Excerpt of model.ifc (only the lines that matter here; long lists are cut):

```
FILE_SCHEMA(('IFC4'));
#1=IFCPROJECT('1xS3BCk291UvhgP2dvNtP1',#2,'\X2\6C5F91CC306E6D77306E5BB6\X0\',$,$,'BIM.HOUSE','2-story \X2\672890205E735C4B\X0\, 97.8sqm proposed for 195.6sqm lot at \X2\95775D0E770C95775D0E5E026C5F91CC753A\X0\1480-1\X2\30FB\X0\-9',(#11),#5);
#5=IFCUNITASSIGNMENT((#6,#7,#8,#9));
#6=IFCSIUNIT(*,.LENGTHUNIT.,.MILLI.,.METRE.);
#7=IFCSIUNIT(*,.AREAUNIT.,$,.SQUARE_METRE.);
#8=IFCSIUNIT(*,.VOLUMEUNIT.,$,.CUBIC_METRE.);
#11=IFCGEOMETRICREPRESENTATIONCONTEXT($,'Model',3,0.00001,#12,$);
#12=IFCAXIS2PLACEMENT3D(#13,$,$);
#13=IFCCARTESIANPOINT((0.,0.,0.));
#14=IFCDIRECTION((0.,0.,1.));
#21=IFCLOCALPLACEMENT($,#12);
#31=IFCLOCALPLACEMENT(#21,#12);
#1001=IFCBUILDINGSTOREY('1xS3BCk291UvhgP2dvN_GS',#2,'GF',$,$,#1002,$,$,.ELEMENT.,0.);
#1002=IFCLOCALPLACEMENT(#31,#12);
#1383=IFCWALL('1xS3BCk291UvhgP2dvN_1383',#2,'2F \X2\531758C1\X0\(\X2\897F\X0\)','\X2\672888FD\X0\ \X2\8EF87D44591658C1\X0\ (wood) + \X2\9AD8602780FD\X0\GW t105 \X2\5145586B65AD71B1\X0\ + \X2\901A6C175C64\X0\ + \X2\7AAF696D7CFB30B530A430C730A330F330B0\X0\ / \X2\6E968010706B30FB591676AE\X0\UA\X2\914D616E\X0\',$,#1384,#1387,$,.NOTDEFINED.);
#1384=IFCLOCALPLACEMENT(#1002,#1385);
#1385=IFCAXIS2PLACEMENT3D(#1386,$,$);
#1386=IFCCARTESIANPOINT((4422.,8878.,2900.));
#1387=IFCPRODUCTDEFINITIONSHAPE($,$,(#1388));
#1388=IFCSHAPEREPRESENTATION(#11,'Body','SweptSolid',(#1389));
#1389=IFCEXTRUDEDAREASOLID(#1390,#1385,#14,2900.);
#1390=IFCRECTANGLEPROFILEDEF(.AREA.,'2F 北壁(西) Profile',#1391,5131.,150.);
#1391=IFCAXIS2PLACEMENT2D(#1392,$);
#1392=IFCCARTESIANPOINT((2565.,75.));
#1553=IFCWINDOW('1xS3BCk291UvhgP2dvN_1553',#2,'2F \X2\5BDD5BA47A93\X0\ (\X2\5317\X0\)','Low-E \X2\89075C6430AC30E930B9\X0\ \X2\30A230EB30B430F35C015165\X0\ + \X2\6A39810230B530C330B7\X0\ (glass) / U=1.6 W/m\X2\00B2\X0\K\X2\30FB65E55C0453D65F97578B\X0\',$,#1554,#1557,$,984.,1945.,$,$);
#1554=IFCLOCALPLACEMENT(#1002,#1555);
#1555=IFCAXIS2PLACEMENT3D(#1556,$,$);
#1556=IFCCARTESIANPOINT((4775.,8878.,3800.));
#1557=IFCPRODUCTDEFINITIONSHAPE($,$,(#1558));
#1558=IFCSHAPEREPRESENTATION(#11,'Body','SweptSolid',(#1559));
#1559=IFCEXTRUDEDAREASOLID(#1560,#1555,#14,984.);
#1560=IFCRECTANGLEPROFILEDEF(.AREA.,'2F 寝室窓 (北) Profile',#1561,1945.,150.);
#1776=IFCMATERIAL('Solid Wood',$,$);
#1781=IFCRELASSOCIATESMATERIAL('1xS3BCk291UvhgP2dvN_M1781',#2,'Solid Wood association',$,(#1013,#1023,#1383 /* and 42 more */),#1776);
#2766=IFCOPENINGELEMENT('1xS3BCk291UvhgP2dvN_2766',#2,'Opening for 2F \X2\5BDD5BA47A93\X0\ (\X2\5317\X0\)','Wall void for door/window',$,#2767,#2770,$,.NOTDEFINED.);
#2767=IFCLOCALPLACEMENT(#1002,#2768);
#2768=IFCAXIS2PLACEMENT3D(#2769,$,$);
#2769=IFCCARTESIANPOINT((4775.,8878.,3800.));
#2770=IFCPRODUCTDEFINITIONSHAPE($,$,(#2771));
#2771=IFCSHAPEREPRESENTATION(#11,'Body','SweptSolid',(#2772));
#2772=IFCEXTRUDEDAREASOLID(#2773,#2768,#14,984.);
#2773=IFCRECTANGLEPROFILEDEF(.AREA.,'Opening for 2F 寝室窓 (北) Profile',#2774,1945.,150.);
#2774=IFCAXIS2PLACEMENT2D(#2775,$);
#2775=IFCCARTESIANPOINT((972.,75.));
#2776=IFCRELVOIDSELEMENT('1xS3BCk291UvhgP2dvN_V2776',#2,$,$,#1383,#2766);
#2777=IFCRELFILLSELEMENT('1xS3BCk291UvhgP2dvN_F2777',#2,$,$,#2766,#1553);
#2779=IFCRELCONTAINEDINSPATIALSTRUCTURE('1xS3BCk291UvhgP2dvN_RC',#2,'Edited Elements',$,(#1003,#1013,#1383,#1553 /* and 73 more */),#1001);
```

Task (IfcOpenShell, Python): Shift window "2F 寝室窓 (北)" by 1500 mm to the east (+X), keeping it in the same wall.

```python
import ifcopenshell
import ifcopenshell.api.geometry
import ifcopenshell.util.placement
import ifcopenshell.util.unit

model = ifcopenshell.open("model.ifc")
unit_scale = ifcopenshell.util.unit.calculate_unit_scale(model)

window = model.by_guid("1xS3BCk291UvhgP2dvN_1553")
opening = window.FillsVoids[0].RelatingOpeningElement
wall = opening.VoidsElements[0].RelatingBuildingElement

wall_matrix = ifcopenshell.util.placement.get_local_placement(wall.ObjectPlacement)
shift = wall_matrix[:3, 0] * 1.5 / unit_scale
before = ifcopenshell.util.placement.get_local_placement(window.ObjectPlacement)[:3, 3].copy()

# The window is not placed relative to its opening, so move both.
for product in (opening, window):
    matrix = ifcopenshell.util.placement.get_local_placement(product.ObjectPlacement)
    matrix[:3, 3] += shift
    ifcopenshell.api.geometry.edit_object_placement(model, product=product, matrix=matrix, is_si=False)

after = ifcopenshell.util.placement.get_local_placement(window.ObjectPlacement)[:3, 3]
print("window moved by", (after - before).round(3) + 0.0)

model.write("model_v2.ifc")
```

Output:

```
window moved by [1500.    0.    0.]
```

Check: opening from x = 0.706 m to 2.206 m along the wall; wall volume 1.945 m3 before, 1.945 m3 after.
